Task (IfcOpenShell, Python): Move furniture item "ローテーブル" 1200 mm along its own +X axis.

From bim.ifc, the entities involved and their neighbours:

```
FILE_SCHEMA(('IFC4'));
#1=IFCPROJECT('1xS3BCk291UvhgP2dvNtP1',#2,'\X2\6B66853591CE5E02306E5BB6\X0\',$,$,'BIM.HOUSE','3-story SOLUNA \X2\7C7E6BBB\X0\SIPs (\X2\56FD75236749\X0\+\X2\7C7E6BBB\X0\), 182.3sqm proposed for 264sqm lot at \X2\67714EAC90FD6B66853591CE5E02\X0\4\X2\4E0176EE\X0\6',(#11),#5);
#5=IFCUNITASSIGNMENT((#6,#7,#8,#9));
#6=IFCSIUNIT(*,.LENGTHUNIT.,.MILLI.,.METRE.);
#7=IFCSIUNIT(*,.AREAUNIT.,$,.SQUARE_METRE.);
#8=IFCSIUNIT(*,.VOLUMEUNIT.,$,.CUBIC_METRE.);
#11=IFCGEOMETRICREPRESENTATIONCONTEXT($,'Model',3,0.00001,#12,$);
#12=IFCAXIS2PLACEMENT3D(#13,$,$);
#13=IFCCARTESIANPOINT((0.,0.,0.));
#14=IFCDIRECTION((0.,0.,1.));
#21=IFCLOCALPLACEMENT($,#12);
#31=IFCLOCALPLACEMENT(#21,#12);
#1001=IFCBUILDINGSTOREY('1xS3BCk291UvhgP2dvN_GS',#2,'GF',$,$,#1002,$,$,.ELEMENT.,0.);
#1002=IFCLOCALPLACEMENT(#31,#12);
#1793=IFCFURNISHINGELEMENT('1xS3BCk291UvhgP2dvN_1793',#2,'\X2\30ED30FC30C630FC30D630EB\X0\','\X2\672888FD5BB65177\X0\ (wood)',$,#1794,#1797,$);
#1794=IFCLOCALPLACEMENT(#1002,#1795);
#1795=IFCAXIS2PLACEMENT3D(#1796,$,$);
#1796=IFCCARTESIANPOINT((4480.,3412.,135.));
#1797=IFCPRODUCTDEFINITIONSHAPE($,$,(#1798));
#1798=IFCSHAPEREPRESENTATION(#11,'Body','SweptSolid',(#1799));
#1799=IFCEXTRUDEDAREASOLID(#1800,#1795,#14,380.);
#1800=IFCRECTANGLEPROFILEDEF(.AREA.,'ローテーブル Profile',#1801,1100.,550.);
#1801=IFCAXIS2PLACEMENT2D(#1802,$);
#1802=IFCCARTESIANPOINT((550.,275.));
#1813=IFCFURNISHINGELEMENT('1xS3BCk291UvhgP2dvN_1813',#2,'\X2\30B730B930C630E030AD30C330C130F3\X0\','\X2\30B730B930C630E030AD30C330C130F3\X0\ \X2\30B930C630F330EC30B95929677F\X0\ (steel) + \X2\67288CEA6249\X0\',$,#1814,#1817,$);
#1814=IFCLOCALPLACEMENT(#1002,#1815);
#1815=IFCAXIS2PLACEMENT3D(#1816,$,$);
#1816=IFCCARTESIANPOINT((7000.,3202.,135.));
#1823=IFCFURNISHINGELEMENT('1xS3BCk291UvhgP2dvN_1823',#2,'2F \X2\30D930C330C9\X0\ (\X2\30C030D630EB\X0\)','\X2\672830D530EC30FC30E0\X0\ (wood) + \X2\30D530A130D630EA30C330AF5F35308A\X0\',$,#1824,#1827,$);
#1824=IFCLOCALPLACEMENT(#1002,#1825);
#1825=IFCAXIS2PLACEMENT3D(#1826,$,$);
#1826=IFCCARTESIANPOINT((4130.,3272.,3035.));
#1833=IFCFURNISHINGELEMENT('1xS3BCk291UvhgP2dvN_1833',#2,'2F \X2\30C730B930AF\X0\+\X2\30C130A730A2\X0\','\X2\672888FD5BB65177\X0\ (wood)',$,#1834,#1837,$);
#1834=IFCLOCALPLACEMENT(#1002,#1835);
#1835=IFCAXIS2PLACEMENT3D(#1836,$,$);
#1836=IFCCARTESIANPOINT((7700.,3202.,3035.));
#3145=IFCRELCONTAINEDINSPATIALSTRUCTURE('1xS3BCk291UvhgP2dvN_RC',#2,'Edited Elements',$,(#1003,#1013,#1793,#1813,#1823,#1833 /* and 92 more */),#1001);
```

```python
import ifcopenshell
import ifcopenshell.api.geometry
import ifcopenshell.util.placement
import ifcopenshell.util.unit

model = ifcopenshell.open("bim.ifc")
unit_scale = ifcopenshell.util.unit.calculate_unit_scale(model)

item = model.by_id(1793)
matrix = ifcopenshell.util.placement.get_local_placement(item.ObjectPlacement)
matrix[:3, 3] += matrix[:3, 0] * 1.2 / unit_scale
ifcopenshell.api.geometry.edit_object_placement(model, product=item, matrix=matrix, is_si=False)

print(ifcopenshell.util.placement.get_local_placement(item.ObjectPlacement).round(3) + 0.0)

model.write("bim-out.ifc")
```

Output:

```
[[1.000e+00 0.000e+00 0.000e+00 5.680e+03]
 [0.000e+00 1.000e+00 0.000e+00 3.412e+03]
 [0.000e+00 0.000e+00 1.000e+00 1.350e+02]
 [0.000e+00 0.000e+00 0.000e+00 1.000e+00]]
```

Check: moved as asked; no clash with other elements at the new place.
